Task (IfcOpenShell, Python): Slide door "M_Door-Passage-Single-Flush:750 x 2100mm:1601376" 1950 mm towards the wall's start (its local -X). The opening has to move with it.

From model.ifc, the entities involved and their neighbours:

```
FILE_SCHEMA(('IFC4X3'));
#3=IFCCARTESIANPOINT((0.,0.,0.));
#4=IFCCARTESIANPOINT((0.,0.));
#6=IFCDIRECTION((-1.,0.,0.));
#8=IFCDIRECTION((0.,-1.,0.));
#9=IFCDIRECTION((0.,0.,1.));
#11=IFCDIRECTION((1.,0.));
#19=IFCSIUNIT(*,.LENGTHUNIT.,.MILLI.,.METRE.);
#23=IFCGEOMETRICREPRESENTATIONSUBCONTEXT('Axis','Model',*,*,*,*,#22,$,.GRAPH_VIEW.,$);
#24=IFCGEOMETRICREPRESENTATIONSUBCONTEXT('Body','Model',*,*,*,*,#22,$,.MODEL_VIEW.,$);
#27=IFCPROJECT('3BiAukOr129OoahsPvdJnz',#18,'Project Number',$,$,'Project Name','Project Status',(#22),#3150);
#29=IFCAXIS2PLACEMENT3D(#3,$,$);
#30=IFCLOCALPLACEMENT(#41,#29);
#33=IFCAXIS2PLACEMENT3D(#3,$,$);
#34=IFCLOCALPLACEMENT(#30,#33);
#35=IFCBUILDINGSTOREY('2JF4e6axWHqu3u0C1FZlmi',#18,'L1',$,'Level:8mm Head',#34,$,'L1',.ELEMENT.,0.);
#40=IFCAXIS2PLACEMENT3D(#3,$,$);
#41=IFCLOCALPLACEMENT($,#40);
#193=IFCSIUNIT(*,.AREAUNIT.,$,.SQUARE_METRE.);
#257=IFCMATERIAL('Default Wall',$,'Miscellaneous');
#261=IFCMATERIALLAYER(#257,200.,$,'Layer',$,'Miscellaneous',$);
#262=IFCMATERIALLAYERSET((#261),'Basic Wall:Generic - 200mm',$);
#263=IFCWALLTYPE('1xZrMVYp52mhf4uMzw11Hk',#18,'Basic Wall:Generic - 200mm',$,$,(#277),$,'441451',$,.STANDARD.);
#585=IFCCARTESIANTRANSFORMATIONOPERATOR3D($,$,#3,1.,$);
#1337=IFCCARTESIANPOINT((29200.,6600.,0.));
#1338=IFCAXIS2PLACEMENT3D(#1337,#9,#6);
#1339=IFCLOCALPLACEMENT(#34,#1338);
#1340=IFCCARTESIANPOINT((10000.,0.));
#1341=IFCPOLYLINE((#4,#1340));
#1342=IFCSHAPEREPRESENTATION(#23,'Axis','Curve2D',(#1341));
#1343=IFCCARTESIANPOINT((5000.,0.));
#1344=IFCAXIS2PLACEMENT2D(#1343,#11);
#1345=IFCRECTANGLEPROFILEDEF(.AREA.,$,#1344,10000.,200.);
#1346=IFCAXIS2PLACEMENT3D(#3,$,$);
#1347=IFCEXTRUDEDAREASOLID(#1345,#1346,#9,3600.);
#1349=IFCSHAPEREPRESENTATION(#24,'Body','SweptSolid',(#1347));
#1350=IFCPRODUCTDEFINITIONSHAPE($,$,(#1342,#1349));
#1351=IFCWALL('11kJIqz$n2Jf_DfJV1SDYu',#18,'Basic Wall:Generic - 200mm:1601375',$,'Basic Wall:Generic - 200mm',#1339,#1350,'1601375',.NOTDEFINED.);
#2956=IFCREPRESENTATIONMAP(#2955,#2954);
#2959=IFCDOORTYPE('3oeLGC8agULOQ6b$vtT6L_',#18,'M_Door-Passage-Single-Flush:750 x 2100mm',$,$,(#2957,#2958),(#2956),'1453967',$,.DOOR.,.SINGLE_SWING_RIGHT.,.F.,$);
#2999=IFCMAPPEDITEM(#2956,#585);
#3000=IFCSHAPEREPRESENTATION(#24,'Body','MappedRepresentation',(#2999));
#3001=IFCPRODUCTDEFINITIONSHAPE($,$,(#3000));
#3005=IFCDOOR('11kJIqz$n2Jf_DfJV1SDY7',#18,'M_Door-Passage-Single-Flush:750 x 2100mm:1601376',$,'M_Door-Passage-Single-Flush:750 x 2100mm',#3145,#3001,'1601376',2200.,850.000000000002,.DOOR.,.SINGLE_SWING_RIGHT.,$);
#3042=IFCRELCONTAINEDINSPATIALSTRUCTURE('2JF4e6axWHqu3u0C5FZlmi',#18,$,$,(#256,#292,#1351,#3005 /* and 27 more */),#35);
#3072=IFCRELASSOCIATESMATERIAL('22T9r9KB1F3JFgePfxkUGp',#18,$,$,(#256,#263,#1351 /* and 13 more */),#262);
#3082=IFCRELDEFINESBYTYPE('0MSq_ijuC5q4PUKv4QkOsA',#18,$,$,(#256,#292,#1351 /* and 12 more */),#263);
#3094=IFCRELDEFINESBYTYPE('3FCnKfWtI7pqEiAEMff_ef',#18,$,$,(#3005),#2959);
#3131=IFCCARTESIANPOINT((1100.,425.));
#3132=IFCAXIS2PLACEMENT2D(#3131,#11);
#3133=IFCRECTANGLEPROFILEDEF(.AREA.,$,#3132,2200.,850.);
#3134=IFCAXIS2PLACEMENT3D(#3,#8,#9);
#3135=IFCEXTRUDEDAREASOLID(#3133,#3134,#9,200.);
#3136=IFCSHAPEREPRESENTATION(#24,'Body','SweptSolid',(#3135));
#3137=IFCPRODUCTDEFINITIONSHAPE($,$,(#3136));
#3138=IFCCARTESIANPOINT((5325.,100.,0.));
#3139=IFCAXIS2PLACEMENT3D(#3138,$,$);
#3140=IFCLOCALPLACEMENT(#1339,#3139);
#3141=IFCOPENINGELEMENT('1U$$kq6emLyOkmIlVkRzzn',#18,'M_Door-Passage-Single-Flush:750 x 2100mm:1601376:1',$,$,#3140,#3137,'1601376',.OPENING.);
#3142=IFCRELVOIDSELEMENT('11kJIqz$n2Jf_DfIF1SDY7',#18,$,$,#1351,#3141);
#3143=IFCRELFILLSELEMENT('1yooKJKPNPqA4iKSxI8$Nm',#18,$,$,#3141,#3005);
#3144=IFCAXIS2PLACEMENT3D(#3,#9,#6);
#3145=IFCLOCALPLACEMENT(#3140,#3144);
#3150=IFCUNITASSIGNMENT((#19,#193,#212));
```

```python
import ifcopenshell
import ifcopenshell.api.geometry
import ifcopenshell.util.placement
import ifcopenshell.util.unit

model = ifcopenshell.open("model.ifc")
unit_scale = ifcopenshell.util.unit.calculate_unit_scale(model)

door = model.by_id(3005)
opening = door.FillsVoids[0].RelatingOpeningElement
wall = opening.VoidsElements[0].RelatingBuildingElement

wall_matrix = ifcopenshell.util.placement.get_local_placement(wall.ObjectPlacement)
shift = wall_matrix[:3, 0] * -1.95 / unit_scale
before = ifcopenshell.util.placement.get_local_placement(door.ObjectPlacement)[:3, 3].copy()

# The door is placed relative to its opening, so it follows when the opening moves.
matrix = ifcopenshell.util.placement.get_local_placement(opening.ObjectPlacement)
matrix[:3, 3] += shift
ifcopenshell.api.geometry.edit_object_placement(
    model, product=opening, matrix=matrix, is_si=False, should_transform_children=True
)

after = ifcopenshell.util.placement.get_local_placement(door.ObjectPlacement)[:3, 3]
print("door moved by", (after - before).round(3) + 0.0)

model.write("model_rev.ifc")
```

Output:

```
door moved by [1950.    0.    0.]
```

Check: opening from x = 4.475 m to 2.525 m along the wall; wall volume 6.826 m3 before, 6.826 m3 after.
